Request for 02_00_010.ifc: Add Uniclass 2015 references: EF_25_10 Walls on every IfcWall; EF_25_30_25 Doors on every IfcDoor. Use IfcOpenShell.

First a look at what the model holds.

```python
import ifcopenshell

model = ifcopenshell.open("02_00_010.ifc")
print(model.schema)
print("classifications:", [c.Name for c in model.by_type("IfcClassification")])
for ifc_class in ("IfcDoor", "IfcRoof", "IfcStair", "IfcWall", "IfcWindow"):
    print(ifc_class, len(model.by_type(ifc_class)))
```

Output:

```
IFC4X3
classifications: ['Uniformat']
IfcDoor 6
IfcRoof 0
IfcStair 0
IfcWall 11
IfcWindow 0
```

```python
import ifcopenshell
import ifcopenshell.api.classification

model = ifcopenshell.open("02_00_010.ifc")

system = ifcopenshell.api.classification.add_classification(model, classification="Uniclass 2015")

codes = {
    "IfcWall": ("EF_25_10", "Walls"),
    "IfcDoor": ("EF_25_30_25", "Doors"),
}
for ifc_class, (code, name) in codes.items():
    products = model.by_type(ifc_class)
    ifcopenshell.api.classification.add_reference(
        model, products=products, classification=system, identification=code, name=name
    )
    print(code, len(products))

model.write("02_00_010_rev.ifc")
```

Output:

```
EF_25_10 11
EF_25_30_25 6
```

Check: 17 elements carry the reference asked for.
